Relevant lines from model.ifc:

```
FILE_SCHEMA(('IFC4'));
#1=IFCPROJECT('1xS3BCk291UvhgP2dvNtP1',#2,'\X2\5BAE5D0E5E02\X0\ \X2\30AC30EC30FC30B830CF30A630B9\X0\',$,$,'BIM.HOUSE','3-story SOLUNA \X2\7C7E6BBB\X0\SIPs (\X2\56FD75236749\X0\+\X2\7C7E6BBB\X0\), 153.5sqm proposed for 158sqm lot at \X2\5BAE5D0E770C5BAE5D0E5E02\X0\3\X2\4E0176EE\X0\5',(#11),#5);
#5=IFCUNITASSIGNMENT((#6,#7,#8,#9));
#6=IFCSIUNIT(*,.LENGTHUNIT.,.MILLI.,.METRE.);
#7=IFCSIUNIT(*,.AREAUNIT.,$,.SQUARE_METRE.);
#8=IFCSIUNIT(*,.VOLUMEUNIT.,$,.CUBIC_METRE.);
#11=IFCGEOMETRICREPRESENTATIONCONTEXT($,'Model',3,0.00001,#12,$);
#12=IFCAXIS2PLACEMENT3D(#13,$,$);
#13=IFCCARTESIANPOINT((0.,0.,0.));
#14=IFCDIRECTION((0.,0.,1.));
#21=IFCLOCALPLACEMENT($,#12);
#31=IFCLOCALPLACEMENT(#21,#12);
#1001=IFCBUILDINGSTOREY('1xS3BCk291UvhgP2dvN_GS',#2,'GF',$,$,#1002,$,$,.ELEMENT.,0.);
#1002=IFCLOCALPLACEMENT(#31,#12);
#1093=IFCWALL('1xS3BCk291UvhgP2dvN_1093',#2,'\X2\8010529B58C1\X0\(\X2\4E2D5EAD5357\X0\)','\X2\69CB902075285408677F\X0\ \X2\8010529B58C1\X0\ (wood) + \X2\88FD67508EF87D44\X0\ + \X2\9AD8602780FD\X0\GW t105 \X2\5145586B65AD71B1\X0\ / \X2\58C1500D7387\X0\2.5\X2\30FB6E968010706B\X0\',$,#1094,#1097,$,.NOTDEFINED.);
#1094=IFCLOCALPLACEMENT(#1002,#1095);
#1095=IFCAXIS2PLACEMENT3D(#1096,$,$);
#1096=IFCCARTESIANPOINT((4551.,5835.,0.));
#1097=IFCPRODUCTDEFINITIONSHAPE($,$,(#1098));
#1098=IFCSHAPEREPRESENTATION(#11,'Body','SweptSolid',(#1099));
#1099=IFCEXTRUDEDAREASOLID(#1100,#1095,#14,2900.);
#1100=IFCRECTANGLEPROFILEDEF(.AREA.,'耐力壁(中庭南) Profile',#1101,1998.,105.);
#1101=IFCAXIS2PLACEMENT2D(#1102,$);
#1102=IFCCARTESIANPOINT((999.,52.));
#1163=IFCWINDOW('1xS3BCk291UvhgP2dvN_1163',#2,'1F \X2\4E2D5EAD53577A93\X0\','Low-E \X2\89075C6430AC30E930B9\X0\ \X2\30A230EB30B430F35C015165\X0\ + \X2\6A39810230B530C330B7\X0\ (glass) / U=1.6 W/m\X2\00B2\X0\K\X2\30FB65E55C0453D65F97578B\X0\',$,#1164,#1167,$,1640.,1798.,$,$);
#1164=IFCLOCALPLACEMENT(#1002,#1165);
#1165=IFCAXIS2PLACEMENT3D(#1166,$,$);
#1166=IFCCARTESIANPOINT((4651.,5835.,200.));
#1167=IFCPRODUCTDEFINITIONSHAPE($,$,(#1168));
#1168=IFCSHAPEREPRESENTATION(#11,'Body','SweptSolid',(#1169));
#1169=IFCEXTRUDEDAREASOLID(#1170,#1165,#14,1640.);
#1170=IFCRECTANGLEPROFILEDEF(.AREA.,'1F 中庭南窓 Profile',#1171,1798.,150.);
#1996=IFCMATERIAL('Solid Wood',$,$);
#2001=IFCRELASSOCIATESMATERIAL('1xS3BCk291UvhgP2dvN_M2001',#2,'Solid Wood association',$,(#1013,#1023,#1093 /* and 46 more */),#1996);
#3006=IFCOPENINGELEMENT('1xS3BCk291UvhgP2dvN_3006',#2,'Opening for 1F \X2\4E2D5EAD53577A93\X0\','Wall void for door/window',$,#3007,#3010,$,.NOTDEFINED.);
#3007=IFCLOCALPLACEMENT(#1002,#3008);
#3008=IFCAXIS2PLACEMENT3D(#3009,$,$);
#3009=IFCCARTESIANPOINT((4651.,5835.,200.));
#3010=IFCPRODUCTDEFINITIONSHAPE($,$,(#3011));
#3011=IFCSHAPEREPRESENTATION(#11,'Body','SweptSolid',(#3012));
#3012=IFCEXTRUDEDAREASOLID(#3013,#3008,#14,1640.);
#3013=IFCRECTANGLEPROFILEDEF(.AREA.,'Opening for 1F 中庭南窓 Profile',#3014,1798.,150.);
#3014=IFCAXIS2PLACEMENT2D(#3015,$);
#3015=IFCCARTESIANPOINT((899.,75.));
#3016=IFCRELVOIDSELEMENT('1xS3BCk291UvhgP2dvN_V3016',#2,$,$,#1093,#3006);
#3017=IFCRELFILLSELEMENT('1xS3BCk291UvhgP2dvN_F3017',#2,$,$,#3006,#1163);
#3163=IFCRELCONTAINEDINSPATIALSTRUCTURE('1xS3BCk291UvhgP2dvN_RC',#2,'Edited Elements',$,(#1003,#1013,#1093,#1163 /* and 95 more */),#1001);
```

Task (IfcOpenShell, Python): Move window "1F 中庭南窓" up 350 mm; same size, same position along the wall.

```python
import numpy as np
import ifcopenshell
import ifcopenshell.api.geometry
import ifcopenshell.util.placement
import ifcopenshell.util.unit

model = ifcopenshell.open("model.ifc")
unit_scale = ifcopenshell.util.unit.calculate_unit_scale(model)

window = model.by_guid("1xS3BCk291UvhgP2dvN_1163")
opening = window.FillsVoids[0].RelatingOpeningElement
dz = 0.35 / unit_scale

shift = np.array([0.0, 0.0, dz])
# The window is not placed relative to its opening, so move both.
for product in (opening, window):
    matrix = ifcopenshell.util.placement.get_local_placement(product.ObjectPlacement)
    matrix[:3, 3] += shift
    ifcopenshell.api.geometry.edit_object_placement(model, product=product, matrix=matrix, is_si=False)

print(f"moved by {dz * unit_scale:+.3f} m")

model.write("model_rev.ifc")
```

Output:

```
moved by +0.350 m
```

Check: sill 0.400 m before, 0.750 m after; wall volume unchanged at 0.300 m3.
